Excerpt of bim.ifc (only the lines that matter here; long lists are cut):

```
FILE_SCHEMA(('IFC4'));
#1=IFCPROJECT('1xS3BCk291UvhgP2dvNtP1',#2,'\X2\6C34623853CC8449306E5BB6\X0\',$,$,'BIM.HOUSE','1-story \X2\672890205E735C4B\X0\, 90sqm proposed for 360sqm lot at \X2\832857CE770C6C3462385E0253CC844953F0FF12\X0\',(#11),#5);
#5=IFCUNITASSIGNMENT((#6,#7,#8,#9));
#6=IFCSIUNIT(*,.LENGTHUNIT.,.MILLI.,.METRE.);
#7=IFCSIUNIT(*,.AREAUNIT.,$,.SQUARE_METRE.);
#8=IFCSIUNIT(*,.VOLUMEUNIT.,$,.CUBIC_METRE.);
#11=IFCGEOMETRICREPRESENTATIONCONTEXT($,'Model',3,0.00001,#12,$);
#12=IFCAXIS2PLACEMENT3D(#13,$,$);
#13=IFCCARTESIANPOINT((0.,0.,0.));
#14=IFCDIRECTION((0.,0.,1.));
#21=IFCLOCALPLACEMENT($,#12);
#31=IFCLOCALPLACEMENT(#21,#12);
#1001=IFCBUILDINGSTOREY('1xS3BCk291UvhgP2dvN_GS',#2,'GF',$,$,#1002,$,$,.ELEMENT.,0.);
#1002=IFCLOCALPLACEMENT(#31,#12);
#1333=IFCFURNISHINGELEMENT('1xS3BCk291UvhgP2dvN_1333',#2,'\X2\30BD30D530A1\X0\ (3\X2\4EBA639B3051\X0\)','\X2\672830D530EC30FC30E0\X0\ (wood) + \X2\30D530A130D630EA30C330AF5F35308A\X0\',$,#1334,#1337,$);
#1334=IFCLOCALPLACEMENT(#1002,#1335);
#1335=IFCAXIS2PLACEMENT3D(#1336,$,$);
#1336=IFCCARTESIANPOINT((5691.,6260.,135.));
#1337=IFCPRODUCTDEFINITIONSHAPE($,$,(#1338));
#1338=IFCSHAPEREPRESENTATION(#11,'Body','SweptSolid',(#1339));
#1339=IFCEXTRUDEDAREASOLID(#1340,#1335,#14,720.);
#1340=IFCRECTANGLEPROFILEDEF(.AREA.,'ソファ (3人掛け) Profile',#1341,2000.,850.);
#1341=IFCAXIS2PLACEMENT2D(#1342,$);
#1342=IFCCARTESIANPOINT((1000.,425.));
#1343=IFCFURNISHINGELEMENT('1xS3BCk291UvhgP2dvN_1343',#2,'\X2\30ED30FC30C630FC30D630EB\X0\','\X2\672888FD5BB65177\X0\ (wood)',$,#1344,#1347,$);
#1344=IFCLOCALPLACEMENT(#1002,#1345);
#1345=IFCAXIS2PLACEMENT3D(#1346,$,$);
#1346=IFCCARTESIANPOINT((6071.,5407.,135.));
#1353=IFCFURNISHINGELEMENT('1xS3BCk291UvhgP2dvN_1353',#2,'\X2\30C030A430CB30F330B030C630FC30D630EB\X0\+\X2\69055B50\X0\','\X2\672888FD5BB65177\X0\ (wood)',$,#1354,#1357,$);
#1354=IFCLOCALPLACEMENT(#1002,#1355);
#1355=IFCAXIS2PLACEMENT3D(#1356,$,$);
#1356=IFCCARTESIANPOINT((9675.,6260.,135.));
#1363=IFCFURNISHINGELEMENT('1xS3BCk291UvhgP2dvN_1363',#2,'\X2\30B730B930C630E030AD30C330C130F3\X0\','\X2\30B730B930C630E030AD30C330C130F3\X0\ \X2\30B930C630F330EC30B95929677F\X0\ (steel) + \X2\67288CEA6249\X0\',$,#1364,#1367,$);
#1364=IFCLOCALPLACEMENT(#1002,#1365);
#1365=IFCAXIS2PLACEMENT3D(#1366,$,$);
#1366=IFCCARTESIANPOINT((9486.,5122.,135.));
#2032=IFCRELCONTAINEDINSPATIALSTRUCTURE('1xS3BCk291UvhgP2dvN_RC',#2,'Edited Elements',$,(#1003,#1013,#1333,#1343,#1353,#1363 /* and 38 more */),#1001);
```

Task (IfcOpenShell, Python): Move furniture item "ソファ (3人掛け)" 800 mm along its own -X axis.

```python
import ifcopenshell
import ifcopenshell.api.geometry
import ifcopenshell.util.placement
import ifcopenshell.util.unit

model = ifcopenshell.open("bim.ifc")
unit_scale = ifcopenshell.util.unit.calculate_unit_scale(model)

item = model.by_guid("1xS3BCk291UvhgP2dvN_1333")
matrix = ifcopenshell.util.placement.get_local_placement(item.ObjectPlacement)
matrix[:3, 3] -= matrix[:3, 0] * 0.8 / unit_scale
ifcopenshell.api.geometry.edit_object_placement(model, product=item, matrix=matrix, is_si=False)

print(ifcopenshell.util.placement.get_local_placement(item.ObjectPlacement).round(3) + 0.0)

model.write("bim_edited.ifc")
```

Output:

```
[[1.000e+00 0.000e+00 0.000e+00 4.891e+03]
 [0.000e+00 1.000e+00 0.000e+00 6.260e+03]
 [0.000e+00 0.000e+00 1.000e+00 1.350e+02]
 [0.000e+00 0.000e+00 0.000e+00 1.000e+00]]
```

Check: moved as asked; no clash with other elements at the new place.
